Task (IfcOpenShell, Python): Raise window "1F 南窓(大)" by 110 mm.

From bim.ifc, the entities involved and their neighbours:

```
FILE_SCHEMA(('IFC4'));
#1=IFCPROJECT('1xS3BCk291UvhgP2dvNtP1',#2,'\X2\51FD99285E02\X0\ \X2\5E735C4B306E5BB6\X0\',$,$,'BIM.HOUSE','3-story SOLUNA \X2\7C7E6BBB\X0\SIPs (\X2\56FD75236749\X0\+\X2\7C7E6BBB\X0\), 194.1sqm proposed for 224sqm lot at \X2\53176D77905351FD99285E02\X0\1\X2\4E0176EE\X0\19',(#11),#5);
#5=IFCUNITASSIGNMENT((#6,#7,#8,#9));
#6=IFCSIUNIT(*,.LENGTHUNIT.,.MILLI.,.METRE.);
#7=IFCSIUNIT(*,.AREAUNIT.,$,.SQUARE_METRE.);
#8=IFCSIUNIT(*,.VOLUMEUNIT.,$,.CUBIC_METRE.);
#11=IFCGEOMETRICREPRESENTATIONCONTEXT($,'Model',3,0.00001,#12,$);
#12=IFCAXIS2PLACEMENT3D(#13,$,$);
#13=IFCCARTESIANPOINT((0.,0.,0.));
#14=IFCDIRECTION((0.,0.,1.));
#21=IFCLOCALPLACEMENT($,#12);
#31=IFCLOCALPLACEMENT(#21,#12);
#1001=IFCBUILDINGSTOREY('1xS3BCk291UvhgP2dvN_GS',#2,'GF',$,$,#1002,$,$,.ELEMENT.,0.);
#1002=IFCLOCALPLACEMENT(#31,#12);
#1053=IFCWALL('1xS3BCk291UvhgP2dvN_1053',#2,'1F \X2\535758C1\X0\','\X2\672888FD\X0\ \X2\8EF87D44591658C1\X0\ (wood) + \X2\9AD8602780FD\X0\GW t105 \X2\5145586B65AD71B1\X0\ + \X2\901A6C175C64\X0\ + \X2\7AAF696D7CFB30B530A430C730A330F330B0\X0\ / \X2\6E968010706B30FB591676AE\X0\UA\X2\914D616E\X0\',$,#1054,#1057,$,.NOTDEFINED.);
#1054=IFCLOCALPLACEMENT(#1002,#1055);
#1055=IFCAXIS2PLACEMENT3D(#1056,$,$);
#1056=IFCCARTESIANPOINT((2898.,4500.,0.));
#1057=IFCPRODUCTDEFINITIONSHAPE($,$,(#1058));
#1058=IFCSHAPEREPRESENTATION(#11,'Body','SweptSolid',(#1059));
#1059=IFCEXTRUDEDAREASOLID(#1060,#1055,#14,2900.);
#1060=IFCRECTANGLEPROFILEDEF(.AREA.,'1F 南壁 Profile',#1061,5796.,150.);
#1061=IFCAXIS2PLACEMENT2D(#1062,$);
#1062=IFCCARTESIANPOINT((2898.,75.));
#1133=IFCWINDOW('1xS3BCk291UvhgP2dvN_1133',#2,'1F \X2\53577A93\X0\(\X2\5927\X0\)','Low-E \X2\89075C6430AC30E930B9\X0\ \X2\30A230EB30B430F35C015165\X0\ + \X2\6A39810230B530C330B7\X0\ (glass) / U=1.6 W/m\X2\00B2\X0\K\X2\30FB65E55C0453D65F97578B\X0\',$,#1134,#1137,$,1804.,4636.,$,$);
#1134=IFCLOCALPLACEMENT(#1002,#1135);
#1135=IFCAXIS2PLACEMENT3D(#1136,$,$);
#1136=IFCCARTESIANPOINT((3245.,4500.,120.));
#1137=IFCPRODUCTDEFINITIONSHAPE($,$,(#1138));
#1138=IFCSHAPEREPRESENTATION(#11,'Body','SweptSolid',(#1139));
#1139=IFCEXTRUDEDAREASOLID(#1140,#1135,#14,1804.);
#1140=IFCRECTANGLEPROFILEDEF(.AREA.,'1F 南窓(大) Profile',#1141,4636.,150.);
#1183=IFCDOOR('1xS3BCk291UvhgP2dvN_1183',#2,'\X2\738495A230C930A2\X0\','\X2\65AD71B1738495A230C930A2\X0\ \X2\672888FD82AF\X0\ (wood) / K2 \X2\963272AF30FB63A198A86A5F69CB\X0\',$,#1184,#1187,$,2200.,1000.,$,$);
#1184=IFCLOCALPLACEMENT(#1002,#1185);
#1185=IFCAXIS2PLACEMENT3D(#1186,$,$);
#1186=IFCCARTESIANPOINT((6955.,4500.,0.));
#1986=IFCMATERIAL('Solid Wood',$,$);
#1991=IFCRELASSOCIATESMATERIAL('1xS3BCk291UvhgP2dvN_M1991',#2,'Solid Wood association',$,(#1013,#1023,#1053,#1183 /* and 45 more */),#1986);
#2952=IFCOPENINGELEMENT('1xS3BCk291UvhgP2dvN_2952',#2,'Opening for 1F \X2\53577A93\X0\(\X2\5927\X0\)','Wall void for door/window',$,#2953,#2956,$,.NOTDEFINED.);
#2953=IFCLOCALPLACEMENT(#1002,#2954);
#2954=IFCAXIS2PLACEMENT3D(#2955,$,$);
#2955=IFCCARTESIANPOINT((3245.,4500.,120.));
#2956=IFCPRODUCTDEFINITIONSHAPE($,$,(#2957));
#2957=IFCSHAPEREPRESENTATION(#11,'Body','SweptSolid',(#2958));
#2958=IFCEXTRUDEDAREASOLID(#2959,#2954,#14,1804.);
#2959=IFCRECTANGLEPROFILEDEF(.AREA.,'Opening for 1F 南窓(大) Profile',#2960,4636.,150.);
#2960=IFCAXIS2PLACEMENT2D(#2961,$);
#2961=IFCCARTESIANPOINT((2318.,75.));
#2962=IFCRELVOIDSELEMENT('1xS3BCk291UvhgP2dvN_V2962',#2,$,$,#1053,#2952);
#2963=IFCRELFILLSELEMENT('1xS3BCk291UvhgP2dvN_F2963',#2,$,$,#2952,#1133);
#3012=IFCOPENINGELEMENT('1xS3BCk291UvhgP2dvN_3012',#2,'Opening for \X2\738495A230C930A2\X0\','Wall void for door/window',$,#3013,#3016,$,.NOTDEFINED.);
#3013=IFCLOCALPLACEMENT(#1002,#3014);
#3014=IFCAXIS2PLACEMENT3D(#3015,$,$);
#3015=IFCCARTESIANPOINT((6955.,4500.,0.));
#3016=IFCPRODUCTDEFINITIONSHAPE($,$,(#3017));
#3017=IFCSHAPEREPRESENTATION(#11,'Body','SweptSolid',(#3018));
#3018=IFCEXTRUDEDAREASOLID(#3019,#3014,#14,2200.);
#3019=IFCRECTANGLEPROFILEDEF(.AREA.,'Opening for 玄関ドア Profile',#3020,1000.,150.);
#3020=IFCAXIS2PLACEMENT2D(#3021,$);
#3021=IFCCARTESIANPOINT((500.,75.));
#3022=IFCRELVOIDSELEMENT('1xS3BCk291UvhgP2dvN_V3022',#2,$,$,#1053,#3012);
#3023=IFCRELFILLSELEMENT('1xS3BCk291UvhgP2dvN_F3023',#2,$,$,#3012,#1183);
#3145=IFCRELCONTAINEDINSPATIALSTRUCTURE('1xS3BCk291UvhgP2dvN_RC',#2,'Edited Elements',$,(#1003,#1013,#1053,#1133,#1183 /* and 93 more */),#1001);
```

```python
import numpy as np
import ifcopenshell
import ifcopenshell.api.geometry
import ifcopenshell.util.placement
import ifcopenshell.util.unit

model = ifcopenshell.open("bim.ifc")
unit_scale = ifcopenshell.util.unit.calculate_unit_scale(model)

window = model.by_guid("1xS3BCk291UvhgP2dvN_1133")
opening = window.FillsVoids[0].RelatingOpeningElement
dz = 0.11 / unit_scale

shift = np.array([0.0, 0.0, dz])
# The window is not placed relative to its opening, so move both.
for product in (opening, window):
    matrix = ifcopenshell.util.placement.get_local_placement(product.ObjectPlacement)
    matrix[:3, 3] += shift
    ifcopenshell.api.geometry.edit_object_placement(model, product=product, matrix=matrix, is_si=False)

print(f"moved by {dz * unit_scale:+.3f} m")

model.write("bim_rev.ifc")
```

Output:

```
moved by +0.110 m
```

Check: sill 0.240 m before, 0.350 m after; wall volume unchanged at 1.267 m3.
